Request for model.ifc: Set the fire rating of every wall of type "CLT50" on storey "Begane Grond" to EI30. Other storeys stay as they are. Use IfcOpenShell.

First a look at what the model holds.

```python
import ifcopenshell
import ifcopenshell.util.element

model = ifcopenshell.open("model.ifc")
print(model.schema)
storey = next(s for s in model.by_type("IfcBuildingStorey") if s.Name == "Begane Grond")
walls = [e for e in ifcopenshell.util.element.get_decomposition(storey) if e.is_a("IfcWall")]
seen = {}
for e in walls:
    element_type = ifcopenshell.util.element.get_type(e)
    key = (element_type.Name if element_type != e and element_type else None, ifcopenshell.util.element.get_pset(e, "Pset_WallCommon", "FireRating"))
    seen[key] = seen.get(key, 0) + 1
for (name, value), count in sorted(seen.items(), key=str):
    print(count, "x", name, "|", value)
```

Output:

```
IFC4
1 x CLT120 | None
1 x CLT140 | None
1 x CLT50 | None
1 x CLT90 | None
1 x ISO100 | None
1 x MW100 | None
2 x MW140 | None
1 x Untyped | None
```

```python
import ifcopenshell
import ifcopenshell.api.pset
import ifcopenshell.util.element

model = ifcopenshell.open("model.ifc")

storey = next(s for s in model.by_type("IfcBuildingStorey") if s.Name == "Begane Grond")
walls = [e for e in ifcopenshell.util.element.get_decomposition(storey) if e.is_a("IfcWall")]

count = 0
for e in walls:
    element_type = ifcopenshell.util.element.get_type(e)
    if element_type in (None, e) or element_type.Name != "CLT50":
        continue
    # add_pset returns the element's existing set when there is one.
    pset = ifcopenshell.api.pset.add_pset(model, product=e, name="Pset_WallCommon")
    ifcopenshell.api.pset.edit_pset(model, pset=pset, properties={"FireRating": "EI30"})
    count += 1

print(count, "walls updated")

model.write("model_rev.ifc")
```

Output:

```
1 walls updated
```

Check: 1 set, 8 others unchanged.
